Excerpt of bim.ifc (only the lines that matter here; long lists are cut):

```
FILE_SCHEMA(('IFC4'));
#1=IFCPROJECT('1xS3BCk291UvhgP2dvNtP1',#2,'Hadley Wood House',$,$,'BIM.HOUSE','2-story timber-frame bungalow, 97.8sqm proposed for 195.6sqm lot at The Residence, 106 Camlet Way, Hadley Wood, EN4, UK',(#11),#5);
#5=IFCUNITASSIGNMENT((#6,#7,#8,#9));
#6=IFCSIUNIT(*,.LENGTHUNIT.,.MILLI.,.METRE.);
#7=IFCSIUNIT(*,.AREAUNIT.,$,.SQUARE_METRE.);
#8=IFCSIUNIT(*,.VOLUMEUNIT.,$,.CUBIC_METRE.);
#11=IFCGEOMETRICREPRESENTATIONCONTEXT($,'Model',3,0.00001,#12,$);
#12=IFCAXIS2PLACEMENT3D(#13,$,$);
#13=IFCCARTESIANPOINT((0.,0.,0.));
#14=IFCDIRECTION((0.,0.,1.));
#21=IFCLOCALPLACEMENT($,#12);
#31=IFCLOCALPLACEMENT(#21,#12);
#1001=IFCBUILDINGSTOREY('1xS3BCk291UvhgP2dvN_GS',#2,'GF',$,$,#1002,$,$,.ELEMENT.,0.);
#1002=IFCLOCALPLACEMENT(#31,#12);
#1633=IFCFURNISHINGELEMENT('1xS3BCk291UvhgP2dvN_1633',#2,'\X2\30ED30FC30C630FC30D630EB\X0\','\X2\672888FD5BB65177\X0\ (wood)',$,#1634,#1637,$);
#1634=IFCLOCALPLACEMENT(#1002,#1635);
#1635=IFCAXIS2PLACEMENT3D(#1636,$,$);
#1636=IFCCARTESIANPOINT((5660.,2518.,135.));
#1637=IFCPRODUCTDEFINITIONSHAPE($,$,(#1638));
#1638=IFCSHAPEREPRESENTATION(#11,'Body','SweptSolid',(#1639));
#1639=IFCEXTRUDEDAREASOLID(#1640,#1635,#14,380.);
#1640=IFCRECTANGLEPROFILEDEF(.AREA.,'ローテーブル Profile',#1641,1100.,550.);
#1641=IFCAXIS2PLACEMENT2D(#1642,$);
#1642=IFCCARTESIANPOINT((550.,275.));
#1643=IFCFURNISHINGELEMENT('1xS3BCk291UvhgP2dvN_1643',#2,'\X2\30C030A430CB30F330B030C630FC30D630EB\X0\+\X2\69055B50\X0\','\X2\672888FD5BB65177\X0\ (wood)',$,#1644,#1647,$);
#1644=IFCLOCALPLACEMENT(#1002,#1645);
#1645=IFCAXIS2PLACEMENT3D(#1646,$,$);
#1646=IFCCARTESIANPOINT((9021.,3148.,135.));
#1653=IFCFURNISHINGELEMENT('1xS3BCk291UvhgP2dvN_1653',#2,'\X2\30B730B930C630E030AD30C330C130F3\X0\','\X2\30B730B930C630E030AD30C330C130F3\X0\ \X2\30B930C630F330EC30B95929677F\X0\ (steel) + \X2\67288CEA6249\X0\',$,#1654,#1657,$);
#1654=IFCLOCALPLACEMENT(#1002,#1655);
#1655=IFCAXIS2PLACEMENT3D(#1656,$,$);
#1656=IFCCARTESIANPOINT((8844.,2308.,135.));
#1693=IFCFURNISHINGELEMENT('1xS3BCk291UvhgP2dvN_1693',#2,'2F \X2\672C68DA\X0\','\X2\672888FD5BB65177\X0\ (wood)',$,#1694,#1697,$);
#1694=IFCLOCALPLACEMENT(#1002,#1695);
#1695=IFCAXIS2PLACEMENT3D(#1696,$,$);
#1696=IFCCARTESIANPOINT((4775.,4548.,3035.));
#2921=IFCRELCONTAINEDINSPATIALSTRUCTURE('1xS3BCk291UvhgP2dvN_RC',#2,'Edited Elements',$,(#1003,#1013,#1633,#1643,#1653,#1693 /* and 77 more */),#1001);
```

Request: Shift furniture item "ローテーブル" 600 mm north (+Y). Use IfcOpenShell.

```python
import ifcopenshell
import ifcopenshell.api.geometry
import ifcopenshell.util.placement

model = ifcopenshell.open("bim.ifc")

item = model.by_id(1633)
matrix = ifcopenshell.util.placement.get_local_placement(item.ObjectPlacement)
matrix[1, 3] += 600.0
ifcopenshell.api.geometry.edit_object_placement(model, product=item, matrix=matrix, is_si=False)

print(ifcopenshell.util.placement.get_local_placement(item.ObjectPlacement).round(3) + 0.0)

model.write("bim_updated.ifc")
```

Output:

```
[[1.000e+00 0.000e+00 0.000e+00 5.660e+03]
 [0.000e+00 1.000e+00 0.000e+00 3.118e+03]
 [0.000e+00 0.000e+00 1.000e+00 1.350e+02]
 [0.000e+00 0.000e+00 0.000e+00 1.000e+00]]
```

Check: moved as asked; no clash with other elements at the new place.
